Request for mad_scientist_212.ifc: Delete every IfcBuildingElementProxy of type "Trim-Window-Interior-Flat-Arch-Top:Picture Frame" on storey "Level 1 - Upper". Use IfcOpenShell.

First a look at what the model holds.

```python
import ifcopenshell
import ifcopenshell.util.element

model = ifcopenshell.open("mad_scientist_212.ifc")
print(model.schema)
storey = next(s for s in model.by_type("IfcBuildingStorey") if s.Name == "Level 1 - Upper")
proxies = [e for e in ifcopenshell.util.element.get_decomposition(storey) if e.is_a("IfcBuildingElementProxy")]
seen = {}
for e in proxies:
    element_type = ifcopenshell.util.element.get_type(e)
    name = element_type.Name if element_type not in (None, e) else None
    seen[name] = seen.get(name, 0) + 1
for name, count in sorted(seen.items(), key=str):
    print(count, "x", name)
```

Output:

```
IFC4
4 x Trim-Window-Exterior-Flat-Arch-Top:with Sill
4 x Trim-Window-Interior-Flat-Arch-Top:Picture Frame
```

```python
import ifcopenshell
import ifcopenshell.api.root
import ifcopenshell.util.element

model = ifcopenshell.open("mad_scientist_212.ifc")

storey = next(s for s in model.by_type("IfcBuildingStorey") if s.Name == "Level 1 - Upper")
proxies = [e for e in ifcopenshell.util.element.get_decomposition(storey) if e.is_a("IfcBuildingElementProxy")]
targets = [e for e in proxies if (t := ifcopenshell.util.element.get_type(e)) not in (None, e) and t.Name == "Trim-Window-Interior-Flat-Arch-Top:Picture Frame"]

for e in targets:
    ifcopenshell.api.root.remove_product(model, product=e)
print(len(targets), "removed")

model.write("mad_scientist_212-out.ifc")
```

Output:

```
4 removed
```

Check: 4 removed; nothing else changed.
